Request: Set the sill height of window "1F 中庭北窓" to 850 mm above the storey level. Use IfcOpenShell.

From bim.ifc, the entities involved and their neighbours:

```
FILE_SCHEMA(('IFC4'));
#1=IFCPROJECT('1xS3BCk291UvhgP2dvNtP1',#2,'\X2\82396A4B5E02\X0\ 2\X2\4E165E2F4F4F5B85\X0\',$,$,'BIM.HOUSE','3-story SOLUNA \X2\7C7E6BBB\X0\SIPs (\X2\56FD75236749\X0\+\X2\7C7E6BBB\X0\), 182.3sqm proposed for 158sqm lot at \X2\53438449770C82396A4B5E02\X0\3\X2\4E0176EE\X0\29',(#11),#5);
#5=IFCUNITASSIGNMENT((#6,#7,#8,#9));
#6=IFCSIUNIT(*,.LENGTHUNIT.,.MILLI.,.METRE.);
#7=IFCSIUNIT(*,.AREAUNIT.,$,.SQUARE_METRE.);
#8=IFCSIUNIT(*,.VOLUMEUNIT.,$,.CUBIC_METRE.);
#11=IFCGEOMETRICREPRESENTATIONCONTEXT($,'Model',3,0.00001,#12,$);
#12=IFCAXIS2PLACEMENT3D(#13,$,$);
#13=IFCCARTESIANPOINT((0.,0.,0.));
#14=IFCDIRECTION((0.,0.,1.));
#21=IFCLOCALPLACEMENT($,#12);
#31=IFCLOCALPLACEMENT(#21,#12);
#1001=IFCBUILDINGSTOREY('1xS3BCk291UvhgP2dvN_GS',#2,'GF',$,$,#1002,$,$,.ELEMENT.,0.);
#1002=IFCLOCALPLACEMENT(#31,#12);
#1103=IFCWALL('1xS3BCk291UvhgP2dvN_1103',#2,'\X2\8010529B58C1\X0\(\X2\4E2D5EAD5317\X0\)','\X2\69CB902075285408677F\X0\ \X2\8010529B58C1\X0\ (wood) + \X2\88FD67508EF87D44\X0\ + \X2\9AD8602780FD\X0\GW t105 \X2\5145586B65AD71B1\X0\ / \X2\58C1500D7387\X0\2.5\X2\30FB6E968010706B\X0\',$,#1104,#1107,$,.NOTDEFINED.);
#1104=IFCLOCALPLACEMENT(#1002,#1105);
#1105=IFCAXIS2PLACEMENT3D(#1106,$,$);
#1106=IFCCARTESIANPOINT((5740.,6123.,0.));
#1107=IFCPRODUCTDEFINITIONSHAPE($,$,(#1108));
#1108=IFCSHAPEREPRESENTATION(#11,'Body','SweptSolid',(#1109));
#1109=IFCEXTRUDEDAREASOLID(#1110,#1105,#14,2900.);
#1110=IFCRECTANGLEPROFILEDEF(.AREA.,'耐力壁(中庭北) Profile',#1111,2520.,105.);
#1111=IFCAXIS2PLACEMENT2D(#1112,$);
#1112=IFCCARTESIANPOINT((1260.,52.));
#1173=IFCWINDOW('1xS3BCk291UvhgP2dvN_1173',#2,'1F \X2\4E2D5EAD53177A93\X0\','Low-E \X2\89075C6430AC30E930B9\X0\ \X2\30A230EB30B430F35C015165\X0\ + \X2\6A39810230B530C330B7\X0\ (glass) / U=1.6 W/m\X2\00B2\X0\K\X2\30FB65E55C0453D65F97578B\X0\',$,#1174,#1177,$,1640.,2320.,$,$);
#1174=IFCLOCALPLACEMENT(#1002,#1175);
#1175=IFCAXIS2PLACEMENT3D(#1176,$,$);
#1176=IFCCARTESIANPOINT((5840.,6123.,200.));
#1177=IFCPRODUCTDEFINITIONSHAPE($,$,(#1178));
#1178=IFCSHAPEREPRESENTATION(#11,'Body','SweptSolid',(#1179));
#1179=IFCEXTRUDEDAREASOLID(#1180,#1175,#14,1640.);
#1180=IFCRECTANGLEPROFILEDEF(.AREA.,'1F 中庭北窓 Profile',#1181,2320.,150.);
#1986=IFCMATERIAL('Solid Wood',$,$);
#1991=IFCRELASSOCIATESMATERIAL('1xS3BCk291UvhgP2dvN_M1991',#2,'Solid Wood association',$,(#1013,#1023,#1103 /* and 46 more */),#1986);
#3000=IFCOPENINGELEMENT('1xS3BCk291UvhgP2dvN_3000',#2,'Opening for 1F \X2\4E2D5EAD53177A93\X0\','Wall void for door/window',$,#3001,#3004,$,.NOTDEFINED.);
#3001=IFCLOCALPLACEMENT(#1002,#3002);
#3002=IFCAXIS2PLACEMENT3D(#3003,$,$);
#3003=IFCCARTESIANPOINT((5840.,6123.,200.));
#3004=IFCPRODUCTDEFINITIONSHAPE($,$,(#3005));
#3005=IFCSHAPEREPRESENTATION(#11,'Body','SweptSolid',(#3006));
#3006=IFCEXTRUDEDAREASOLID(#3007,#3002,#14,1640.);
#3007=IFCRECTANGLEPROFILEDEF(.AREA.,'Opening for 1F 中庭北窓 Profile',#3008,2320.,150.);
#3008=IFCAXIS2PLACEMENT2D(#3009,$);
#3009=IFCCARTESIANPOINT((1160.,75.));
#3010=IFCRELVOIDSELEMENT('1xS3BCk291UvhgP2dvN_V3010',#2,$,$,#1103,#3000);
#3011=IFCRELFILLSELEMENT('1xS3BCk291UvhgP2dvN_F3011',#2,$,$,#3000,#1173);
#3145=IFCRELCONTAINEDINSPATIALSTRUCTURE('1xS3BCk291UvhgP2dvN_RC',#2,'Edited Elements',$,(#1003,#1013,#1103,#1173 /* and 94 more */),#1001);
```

```python
import numpy as np
import ifcopenshell
import ifcopenshell.api.geometry
import ifcopenshell.geom
import ifcopenshell.util.element
import ifcopenshell.util.placement
import ifcopenshell.util.shape
import ifcopenshell.util.unit

model = ifcopenshell.open("bim.ifc")
unit_scale = ifcopenshell.util.unit.calculate_unit_scale(model)

window = model.by_guid("1xS3BCk291UvhgP2dvN_1173")
opening = window.FillsVoids[0].RelatingOpeningElement
storey = ifcopenshell.util.element.get_container(window, ifc_class="IfcBuildingStorey")
level = ifcopenshell.util.placement.get_local_placement(storey.ObjectPlacement)[2, 3]

# The opening's origin need not be at the sill, so measure its lowest point.
shape = ifcopenshell.geom.create_shape(ifcopenshell.geom.settings(), opening)
bottom = ifcopenshell.util.shape.get_shape_bottom_elevation(shape, shape.geometry) / unit_scale
dz = level + 0.85 / unit_scale - bottom

shift = np.array([0.0, 0.0, dz])
# The window is not placed relative to its opening, so move both.
for product in (opening, window):
    matrix = ifcopenshell.util.placement.get_local_placement(product.ObjectPlacement)
    matrix[:3, 3] += shift
    ifcopenshell.api.geometry.edit_object_placement(model, product=product, matrix=matrix, is_si=False)

print(f"moved by {dz * unit_scale:+.3f} m")

model.write("bim_rev.ifc")
```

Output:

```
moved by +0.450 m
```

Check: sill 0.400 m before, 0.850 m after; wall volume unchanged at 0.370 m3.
